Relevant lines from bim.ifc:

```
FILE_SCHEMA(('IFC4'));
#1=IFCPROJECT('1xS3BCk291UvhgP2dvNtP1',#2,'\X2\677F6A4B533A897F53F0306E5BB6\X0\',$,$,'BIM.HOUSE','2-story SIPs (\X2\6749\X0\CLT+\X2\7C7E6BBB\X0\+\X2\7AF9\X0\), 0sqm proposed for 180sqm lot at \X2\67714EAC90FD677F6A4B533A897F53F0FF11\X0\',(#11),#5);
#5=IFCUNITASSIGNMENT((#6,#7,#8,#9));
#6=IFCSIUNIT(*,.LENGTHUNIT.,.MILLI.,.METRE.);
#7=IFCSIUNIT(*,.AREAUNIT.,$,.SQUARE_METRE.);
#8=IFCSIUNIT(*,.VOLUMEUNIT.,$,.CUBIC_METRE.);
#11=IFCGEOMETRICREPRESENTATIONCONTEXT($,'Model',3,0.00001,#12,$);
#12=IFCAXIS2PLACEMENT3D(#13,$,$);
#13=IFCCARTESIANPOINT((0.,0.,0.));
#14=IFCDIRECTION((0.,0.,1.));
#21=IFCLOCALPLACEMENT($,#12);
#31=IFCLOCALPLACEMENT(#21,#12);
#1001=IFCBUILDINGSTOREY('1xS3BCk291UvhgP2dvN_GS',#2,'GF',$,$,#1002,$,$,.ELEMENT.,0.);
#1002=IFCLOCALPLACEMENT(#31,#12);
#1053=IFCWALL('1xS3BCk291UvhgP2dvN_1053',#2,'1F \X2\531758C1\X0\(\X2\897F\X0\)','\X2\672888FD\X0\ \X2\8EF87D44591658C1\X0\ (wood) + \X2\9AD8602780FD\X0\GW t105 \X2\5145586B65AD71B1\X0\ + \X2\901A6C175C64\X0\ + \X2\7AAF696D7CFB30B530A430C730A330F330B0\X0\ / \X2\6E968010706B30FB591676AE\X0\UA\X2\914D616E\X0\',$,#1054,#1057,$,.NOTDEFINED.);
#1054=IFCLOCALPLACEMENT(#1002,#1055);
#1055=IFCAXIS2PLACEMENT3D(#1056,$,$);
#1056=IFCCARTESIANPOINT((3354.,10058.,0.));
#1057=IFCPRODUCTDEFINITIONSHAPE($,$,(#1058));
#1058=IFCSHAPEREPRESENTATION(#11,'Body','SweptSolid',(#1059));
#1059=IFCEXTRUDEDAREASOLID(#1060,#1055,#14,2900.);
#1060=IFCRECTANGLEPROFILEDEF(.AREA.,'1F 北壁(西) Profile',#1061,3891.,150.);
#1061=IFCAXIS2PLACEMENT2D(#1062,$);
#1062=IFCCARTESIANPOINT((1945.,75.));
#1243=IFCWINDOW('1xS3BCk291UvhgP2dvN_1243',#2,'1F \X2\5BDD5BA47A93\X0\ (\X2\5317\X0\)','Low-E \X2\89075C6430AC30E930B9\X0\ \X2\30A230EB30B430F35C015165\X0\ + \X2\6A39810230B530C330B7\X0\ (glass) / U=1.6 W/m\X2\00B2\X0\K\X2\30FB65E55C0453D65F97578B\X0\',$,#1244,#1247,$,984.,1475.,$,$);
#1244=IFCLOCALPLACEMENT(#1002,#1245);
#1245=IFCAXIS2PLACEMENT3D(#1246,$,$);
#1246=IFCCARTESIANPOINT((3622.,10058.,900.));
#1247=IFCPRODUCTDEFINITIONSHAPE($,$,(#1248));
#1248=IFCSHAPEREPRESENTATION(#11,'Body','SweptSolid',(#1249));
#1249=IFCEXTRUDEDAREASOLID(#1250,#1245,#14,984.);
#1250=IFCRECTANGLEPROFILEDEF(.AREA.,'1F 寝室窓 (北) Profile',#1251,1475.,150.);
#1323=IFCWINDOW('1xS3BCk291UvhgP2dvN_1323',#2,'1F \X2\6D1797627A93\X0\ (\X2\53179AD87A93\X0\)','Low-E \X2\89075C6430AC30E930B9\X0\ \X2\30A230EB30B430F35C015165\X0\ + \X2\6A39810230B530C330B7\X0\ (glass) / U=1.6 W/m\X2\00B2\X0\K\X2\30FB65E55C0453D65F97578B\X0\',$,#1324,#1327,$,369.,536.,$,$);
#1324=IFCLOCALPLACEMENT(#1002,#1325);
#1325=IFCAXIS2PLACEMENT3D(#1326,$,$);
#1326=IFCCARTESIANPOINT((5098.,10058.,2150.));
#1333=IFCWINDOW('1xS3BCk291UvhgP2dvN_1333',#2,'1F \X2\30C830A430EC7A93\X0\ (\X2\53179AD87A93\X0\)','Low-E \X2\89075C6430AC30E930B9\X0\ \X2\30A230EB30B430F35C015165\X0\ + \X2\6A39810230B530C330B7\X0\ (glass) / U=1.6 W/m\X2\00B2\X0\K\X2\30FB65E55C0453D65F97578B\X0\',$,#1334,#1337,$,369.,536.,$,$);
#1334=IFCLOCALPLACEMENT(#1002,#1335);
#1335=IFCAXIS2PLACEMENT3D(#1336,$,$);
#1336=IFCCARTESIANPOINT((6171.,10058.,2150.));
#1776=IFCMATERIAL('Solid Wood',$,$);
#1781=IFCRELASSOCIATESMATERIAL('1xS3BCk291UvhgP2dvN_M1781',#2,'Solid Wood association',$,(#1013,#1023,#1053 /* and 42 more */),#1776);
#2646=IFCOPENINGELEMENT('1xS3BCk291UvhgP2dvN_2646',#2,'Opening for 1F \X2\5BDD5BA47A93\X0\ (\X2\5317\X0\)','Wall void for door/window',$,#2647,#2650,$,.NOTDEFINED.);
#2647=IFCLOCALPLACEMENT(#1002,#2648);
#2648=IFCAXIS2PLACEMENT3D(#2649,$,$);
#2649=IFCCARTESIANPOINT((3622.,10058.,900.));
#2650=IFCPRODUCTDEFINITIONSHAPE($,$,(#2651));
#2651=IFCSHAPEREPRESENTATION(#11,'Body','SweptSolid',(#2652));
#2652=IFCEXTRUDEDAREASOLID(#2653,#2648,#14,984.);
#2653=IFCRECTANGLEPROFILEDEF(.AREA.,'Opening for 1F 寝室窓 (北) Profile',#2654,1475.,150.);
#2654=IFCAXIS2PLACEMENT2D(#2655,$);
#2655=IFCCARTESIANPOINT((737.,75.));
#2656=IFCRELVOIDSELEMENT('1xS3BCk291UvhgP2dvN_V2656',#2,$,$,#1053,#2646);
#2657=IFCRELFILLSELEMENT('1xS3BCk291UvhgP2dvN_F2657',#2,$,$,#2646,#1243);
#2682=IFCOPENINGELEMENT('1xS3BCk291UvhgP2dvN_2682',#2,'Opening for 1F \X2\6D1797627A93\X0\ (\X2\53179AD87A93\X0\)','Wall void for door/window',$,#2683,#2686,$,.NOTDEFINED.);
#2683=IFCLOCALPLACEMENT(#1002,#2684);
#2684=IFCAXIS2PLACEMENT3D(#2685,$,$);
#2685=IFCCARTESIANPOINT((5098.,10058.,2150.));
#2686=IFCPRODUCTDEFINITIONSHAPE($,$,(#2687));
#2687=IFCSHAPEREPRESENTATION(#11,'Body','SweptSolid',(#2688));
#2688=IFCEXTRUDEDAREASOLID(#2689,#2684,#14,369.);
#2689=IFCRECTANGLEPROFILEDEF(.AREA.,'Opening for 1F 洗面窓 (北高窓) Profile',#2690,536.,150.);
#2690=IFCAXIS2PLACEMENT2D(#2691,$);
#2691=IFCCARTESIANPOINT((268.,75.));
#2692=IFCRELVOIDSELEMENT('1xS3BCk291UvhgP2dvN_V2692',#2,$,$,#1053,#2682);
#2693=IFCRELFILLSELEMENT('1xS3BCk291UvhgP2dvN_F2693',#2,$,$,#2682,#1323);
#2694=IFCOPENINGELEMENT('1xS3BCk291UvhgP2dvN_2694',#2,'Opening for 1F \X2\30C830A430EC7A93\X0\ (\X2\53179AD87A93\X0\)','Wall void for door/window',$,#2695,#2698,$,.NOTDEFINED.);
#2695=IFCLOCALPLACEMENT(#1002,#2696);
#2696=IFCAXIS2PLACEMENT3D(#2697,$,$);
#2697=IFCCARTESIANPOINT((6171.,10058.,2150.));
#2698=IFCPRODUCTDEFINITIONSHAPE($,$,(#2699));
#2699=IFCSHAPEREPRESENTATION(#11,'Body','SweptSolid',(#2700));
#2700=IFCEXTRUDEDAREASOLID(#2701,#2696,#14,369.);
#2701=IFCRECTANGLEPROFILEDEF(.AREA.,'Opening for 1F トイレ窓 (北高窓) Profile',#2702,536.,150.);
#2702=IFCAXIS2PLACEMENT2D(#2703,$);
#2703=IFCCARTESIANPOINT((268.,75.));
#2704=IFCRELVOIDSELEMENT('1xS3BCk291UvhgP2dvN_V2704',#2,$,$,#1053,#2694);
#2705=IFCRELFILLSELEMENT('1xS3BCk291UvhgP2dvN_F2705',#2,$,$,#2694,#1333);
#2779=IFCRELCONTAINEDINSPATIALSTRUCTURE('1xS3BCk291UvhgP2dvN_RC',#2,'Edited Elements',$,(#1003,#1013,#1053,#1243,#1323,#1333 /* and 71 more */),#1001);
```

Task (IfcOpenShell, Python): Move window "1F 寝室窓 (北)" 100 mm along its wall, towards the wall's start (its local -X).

```python
import ifcopenshell
import ifcopenshell.api.geometry
import ifcopenshell.util.placement
import ifcopenshell.util.unit

model = ifcopenshell.open("bim.ifc")
unit_scale = ifcopenshell.util.unit.calculate_unit_scale(model)

window = model.by_guid("1xS3BCk291UvhgP2dvN_1243")
opening = window.FillsVoids[0].RelatingOpeningElement
wall = opening.VoidsElements[0].RelatingBuildingElement

wall_matrix = ifcopenshell.util.placement.get_local_placement(wall.ObjectPlacement)
shift = wall_matrix[:3, 0] * -0.1 / unit_scale
before = ifcopenshell.util.placement.get_local_placement(window.ObjectPlacement)[:3, 3].copy()

# The window is not placed relative to its opening, so move both.
for product in (opening, window):
    matrix = ifcopenshell.util.placement.get_local_placement(product.ObjectPlacement)
    matrix[:3, 3] += shift
    ifcopenshell.api.geometry.edit_object_placement(model, product=product, matrix=matrix, is_si=False)

after = ifcopenshell.util.placement.get_local_placement(window.ObjectPlacement)[:3, 3]
print("window moved by", (after - before).round(3) + 0.0)

model.write("bim_rev.ifc")
```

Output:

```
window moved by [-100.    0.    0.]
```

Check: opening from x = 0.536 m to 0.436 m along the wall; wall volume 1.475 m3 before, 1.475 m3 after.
